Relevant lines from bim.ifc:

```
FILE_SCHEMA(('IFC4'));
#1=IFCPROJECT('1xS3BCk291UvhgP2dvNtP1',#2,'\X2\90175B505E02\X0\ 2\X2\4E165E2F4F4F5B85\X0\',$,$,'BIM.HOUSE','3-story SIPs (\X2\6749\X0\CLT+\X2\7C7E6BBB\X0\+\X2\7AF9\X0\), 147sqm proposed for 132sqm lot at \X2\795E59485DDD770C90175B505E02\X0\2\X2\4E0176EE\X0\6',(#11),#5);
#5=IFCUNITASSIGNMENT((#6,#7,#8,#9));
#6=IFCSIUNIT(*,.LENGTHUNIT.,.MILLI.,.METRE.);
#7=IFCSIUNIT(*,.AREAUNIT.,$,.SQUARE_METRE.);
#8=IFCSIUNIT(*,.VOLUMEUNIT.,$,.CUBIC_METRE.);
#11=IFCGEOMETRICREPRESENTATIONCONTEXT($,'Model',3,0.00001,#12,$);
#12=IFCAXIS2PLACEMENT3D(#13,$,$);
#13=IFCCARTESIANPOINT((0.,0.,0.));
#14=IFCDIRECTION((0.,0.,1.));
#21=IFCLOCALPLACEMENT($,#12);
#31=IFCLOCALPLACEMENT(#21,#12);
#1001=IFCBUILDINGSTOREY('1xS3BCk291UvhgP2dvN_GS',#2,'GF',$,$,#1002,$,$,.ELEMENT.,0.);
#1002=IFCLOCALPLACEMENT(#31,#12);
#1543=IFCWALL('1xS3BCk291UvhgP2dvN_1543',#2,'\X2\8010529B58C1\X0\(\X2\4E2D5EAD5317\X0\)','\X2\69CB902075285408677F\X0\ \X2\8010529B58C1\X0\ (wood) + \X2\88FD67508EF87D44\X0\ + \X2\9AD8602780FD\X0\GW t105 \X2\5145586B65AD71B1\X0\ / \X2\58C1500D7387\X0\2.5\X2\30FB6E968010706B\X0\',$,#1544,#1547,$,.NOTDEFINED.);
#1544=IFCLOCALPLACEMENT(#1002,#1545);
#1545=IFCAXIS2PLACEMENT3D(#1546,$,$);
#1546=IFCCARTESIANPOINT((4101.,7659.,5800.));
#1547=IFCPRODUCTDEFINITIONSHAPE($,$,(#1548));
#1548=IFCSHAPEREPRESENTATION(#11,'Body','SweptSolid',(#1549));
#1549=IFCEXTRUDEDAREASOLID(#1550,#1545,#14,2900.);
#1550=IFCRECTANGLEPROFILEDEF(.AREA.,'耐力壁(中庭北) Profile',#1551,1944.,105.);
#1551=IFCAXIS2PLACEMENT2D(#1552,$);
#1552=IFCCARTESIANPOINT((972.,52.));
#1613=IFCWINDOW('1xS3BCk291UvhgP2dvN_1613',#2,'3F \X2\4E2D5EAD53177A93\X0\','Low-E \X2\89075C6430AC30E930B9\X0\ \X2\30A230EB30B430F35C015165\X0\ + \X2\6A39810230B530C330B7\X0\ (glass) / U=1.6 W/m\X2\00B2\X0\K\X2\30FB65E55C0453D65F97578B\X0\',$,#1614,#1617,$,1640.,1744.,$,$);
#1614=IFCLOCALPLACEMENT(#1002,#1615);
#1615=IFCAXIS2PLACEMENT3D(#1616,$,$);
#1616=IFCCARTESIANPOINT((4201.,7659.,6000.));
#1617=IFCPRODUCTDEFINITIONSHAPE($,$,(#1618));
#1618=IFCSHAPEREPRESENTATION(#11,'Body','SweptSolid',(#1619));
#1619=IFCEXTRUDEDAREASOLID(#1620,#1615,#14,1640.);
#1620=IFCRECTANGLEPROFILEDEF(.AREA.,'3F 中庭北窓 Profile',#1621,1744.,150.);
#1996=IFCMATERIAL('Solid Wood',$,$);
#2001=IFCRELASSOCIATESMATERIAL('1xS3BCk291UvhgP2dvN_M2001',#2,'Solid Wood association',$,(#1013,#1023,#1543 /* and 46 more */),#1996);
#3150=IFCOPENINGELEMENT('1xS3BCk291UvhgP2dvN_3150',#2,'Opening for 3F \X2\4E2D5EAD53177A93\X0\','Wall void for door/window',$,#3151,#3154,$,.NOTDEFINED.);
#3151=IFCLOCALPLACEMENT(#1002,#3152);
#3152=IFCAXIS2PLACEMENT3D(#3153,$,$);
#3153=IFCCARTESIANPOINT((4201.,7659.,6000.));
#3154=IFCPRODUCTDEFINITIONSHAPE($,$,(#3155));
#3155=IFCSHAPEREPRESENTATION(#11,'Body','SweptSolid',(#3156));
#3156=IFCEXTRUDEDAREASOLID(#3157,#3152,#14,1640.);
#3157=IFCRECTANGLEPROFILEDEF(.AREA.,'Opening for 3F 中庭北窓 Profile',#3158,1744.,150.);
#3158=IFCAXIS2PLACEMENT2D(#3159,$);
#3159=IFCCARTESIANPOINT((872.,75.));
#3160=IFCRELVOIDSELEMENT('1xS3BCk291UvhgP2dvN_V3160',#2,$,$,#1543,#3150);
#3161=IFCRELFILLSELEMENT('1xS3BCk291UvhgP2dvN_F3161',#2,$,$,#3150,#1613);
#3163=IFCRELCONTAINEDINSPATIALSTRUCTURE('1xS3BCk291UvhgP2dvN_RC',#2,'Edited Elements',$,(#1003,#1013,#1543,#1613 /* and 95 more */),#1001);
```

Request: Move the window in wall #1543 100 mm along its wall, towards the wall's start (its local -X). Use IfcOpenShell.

```python
import ifcopenshell
import ifcopenshell.api.geometry
import ifcopenshell.util.placement
import ifcopenshell.util.unit

model = ifcopenshell.open("bim.ifc")
unit_scale = ifcopenshell.util.unit.calculate_unit_scale(model)

window = model.by_id(1613)
opening = window.FillsVoids[0].RelatingOpeningElement
wall = opening.VoidsElements[0].RelatingBuildingElement

wall_matrix = ifcopenshell.util.placement.get_local_placement(wall.ObjectPlacement)
shift = wall_matrix[:3, 0] * -0.1 / unit_scale
before = ifcopenshell.util.placement.get_local_placement(window.ObjectPlacement)[:3, 3].copy()

# The window is not placed relative to its opening, so move both.
for product in (opening, window):
    matrix = ifcopenshell.util.placement.get_local_placement(product.ObjectPlacement)
    matrix[:3, 3] += shift
    ifcopenshell.api.geometry.edit_object_placement(model, product=product, matrix=matrix, is_si=False)

after = ifcopenshell.util.placement.get_local_placement(window.ObjectPlacement)[:3, 3]
print("window moved by", (after - before).round(3) + 0.0)

model.write("bim_edited.ifc")
```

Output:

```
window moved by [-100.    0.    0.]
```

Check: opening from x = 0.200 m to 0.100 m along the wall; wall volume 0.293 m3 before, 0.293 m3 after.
